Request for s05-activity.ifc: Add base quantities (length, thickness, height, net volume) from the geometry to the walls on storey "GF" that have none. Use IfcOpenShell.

First a look at what the model holds.

```python
import ifcopenshell
import ifcopenshell.util.element
import ifcopenshell.util.unit

model = ifcopenshell.open("s05-activity.ifc")
print(model.schema)
for unit_type in ("LENGTHUNIT", "AREAUNIT", "VOLUMEUNIT"):
    print(unit_type, ifcopenshell.util.unit.calculate_unit_scale(model, unit_type))
storey = next(s for s in model.by_type("IfcBuildingStorey") if s.Name == "GF")
walls = [e for e in ifcopenshell.util.element.get_decomposition(storey) if e.is_a("IfcWall")]
for e in sorted(walls, key=lambda e: e.id()):
    print(e.id(), e.is_a(), e.Name, list(ifcopenshell.util.element.get_psets(e, qtos_only=True)), sep=" | ")
```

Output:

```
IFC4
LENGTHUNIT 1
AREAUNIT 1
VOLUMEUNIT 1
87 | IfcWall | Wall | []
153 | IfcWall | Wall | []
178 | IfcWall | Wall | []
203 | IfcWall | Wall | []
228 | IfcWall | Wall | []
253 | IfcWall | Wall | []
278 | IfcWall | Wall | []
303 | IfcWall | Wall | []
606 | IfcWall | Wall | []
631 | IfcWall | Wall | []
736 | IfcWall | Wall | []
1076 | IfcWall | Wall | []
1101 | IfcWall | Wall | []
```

```python
import ifcopenshell
import ifcopenshell.api.pset
import ifcopenshell.geom
import ifcopenshell.util.element
import ifcopenshell.util.shape
import ifcopenshell.util.unit

model = ifcopenshell.open("s05-activity.ifc")
unit_scale = ifcopenshell.util.unit.calculate_unit_scale(model)
volume_scale = ifcopenshell.util.unit.calculate_unit_scale(model, "VOLUMEUNIT")
settings = ifcopenshell.geom.settings()

storey = next(s for s in model.by_type("IfcBuildingStorey") if s.Name == "GF")
walls = [e for e in ifcopenshell.util.element.get_decomposition(storey) if e.is_a("IfcWall")]

for e in sorted(walls, key=lambda e: e.id()):
    if ifcopenshell.util.element.get_psets(e, qtos_only=True, should_inherit=False):
        continue
    # Geometry comes back in metres, in the element's own axes.
    shape = ifcopenshell.geom.create_shape(settings, e)
    values = {
        "Length": ifcopenshell.util.shape.get_x(shape.geometry) / unit_scale,
        "Width": ifcopenshell.util.shape.get_y(shape.geometry) / unit_scale,
        "Height": ifcopenshell.util.shape.get_z(shape.geometry) / unit_scale,
        "NetVolume": ifcopenshell.util.shape.get_volume(shape.geometry) / volume_scale,
    }
    qto = ifcopenshell.api.pset.add_qto(model, product=e, name="Qto_WallBaseQuantities")
    ifcopenshell.api.pset.edit_qto(model, qto=qto, properties=values)
    print(e.id(), {k: round(v, 3) for k, v in values.items()})

model.write("s05-activity_v2.ifc")
```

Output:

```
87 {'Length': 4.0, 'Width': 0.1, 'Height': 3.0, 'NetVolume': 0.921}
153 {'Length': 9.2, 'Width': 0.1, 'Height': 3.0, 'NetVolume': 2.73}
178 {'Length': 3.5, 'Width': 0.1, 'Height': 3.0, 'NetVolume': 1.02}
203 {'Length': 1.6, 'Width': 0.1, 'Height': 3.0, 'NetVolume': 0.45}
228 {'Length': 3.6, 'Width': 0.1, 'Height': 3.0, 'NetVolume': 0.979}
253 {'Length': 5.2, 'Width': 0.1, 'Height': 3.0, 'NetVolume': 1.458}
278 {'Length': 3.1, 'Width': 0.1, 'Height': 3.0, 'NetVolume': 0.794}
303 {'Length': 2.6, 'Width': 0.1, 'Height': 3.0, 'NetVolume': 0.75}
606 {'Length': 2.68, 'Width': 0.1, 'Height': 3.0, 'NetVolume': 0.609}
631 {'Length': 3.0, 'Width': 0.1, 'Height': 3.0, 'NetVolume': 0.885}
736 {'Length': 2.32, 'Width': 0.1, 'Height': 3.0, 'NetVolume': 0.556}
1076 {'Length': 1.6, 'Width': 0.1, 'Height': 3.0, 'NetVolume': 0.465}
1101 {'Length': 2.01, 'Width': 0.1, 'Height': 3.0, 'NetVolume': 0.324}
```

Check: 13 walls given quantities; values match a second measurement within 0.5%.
